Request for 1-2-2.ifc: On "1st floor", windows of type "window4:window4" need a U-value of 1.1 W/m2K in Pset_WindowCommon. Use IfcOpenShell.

First a look at what the model holds.

```python
import ifcopenshell
import ifcopenshell.util.element

model = ifcopenshell.open("1-2-2.ifc")
print(model.schema)
storey = next(s for s in model.by_type("IfcBuildingStorey") if s.Name == "1st floor")
windows = [e for e in ifcopenshell.util.element.get_decomposition(storey) if e.is_a("IfcWindow")]
seen = {}
for e in windows:
    element_type = ifcopenshell.util.element.get_type(e)
    key = (element_type.Name if element_type != e and element_type else None, ifcopenshell.util.element.get_pset(e, "Pset_WindowCommon", "ThermalTransmittance"))
    seen[key] = seen.get(key, 0) + 1
for (name, value), count in sorted(seen.items(), key=str):
    print(count, "x", name, "|", value)
```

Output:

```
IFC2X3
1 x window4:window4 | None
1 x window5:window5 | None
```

```python
import ifcopenshell
import ifcopenshell.api.pset
import ifcopenshell.util.element

model = ifcopenshell.open("1-2-2.ifc")

storey = next(s for s in model.by_type("IfcBuildingStorey") if s.Name == "1st floor")
windows = [e for e in ifcopenshell.util.element.get_decomposition(storey) if e.is_a("IfcWindow")]

count = 0
for e in windows:
    element_type = ifcopenshell.util.element.get_type(e)
    if element_type in (None, e) or element_type.Name != "window4:window4":
        continue
    # add_pset returns the element's existing set when there is one.
    pset = ifcopenshell.api.pset.add_pset(model, product=e, name="Pset_WindowCommon")
    ifcopenshell.api.pset.edit_pset(model, pset=pset, properties={"ThermalTransmittance": 1.1})
    count += 1

print(count, "windows updated")

model.write("1-2-2_v2.ifc")
```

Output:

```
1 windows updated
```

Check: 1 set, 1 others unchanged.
